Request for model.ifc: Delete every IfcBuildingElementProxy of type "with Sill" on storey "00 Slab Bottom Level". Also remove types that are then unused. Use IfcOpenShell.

First a look at what the model holds.

```python
import ifcopenshell
import ifcopenshell.util.element

model = ifcopenshell.open("model.ifc")
print(model.schema)
storey = next(s for s in model.by_type("IfcBuildingStorey") if s.Name == "00 Slab Bottom Level")
proxies = [e for e in ifcopenshell.util.element.get_decomposition(storey) if e.is_a("IfcBuildingElementProxy")]
seen = {}
for e in proxies:
    element_type = ifcopenshell.util.element.get_type(e)
    name = element_type.Name if element_type not in (None, e) else None
    seen[name] = seen.get(name, 0) + 1
for name, count in sorted(seen.items(), key=str):
    print(count, "x", name)
```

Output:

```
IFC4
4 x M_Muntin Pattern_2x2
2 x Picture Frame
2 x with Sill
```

```python
import ifcopenshell
import ifcopenshell.api.root
import ifcopenshell.util.element

model = ifcopenshell.open("model.ifc")

storey = next(s for s in model.by_type("IfcBuildingStorey") if s.Name == "00 Slab Bottom Level")
proxies = [e for e in ifcopenshell.util.element.get_decomposition(storey) if e.is_a("IfcBuildingElementProxy")]
targets = [e for e in proxies if (t := ifcopenshell.util.element.get_type(e)) not in (None, e) and t.Name == "with Sill"]
types = {ifcopenshell.util.element.get_type(e) for e in targets} - {None, *targets}

for e in targets:
    ifcopenshell.api.root.remove_product(model, product=e)
print(len(targets), "removed")

unused = [t for t in types if not ifcopenshell.util.element.get_types(t)]
for t in unused:
    ifcopenshell.api.root.remove_product(model, product=t)
print(len(unused), "unused types removed")

model.write("model_updated.ifc")
```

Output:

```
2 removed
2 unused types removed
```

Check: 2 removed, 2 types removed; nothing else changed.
